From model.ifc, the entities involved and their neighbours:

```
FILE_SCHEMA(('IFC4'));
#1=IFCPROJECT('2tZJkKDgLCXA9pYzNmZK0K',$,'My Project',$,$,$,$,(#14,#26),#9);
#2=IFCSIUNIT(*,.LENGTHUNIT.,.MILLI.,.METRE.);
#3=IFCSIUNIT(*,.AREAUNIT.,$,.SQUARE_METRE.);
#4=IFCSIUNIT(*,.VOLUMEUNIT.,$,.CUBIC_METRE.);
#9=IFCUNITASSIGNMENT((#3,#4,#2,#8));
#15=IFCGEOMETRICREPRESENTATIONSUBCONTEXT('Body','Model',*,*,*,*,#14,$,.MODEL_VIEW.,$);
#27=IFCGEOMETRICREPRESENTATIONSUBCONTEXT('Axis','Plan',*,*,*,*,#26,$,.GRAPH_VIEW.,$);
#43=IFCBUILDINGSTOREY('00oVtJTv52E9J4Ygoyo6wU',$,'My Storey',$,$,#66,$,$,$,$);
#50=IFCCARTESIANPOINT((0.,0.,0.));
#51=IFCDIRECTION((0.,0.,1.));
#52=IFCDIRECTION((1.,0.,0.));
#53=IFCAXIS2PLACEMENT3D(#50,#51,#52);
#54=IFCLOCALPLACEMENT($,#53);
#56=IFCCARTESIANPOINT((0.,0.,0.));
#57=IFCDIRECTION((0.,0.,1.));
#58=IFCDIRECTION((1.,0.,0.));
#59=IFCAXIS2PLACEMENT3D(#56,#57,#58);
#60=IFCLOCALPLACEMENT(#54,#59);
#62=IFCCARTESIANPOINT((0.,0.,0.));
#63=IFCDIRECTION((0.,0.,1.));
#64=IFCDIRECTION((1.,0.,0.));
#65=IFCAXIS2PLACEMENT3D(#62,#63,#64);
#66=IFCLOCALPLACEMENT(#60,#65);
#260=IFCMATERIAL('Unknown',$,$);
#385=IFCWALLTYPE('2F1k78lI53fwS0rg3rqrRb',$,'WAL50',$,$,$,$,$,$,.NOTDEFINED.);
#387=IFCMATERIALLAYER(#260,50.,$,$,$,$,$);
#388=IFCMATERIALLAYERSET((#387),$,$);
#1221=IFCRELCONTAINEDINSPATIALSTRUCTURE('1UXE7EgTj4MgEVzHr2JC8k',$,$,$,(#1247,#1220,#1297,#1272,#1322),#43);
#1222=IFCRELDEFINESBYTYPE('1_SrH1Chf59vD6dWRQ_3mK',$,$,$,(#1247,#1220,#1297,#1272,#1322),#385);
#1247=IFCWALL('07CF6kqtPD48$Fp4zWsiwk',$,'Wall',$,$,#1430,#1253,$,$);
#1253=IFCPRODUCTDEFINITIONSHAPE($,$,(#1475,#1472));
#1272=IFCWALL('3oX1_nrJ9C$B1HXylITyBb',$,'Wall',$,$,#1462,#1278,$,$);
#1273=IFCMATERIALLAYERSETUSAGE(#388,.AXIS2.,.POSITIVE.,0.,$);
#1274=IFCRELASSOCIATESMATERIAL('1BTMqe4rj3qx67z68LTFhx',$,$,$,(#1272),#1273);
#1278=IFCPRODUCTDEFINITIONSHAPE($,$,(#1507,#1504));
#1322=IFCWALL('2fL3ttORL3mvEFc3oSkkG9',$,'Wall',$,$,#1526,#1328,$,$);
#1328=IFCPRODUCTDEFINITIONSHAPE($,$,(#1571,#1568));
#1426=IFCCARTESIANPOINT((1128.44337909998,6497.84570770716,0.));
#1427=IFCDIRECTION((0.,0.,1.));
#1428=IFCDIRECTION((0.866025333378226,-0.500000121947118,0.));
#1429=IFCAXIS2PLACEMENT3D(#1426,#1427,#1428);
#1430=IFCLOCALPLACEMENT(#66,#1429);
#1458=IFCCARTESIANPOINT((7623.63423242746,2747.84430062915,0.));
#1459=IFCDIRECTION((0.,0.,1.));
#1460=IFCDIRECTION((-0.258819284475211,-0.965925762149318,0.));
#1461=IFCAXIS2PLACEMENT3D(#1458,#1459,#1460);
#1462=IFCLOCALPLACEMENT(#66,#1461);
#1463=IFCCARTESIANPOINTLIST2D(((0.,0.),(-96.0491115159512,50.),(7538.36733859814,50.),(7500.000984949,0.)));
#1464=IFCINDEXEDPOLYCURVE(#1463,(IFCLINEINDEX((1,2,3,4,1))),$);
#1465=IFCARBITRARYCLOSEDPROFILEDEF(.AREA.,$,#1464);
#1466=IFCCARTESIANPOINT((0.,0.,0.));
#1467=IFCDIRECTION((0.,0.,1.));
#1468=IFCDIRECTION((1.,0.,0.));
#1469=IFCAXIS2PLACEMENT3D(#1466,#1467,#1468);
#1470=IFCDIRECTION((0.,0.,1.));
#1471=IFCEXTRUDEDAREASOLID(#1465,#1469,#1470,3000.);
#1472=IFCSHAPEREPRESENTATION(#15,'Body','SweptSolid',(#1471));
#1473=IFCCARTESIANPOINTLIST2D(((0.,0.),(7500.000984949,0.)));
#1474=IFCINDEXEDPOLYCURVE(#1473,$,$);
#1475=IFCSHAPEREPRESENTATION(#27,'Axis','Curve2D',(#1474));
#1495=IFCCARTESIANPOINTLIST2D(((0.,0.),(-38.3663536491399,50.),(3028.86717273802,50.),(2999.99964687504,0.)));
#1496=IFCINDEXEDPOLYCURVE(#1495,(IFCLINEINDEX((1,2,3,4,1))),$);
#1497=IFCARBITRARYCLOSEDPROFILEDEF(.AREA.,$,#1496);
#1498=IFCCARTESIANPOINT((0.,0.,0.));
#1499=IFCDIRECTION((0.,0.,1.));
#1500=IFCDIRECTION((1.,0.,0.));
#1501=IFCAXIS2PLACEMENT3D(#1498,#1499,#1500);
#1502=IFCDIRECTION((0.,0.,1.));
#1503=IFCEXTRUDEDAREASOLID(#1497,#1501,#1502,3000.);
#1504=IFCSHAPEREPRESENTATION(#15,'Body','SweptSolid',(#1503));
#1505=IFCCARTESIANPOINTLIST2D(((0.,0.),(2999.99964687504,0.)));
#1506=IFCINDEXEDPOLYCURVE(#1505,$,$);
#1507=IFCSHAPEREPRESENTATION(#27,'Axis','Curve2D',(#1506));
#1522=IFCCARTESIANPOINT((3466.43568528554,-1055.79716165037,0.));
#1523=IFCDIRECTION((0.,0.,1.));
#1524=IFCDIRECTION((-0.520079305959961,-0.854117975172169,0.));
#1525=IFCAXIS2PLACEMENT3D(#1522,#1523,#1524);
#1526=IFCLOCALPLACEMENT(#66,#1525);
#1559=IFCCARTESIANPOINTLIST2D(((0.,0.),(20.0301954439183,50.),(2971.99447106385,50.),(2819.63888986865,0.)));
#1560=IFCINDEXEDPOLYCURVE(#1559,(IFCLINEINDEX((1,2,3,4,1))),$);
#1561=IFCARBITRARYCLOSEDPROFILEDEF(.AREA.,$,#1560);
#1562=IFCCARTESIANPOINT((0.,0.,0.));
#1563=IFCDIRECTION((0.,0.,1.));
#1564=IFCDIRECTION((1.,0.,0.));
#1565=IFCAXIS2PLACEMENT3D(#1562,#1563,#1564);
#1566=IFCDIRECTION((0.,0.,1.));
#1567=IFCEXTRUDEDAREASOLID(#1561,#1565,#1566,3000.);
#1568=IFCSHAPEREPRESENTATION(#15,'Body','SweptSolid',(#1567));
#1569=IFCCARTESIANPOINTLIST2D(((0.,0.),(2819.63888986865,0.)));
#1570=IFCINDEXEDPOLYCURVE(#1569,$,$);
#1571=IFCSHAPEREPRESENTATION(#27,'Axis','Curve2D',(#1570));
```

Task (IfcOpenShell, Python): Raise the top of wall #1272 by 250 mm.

```python
import ifcopenshell
import ifcopenshell.geom
import ifcopenshell.util.representation
import ifcopenshell.util.shape
import ifcopenshell.util.unit

model = ifcopenshell.open("model.ifc")
unit_scale = ifcopenshell.util.unit.calculate_unit_scale(model)
settings = ifcopenshell.geom.settings()


def volume(element):
    """Net volume in cubic metres, openings subtracted."""
    shape = ifcopenshell.geom.create_shape(settings, element)
    return ifcopenshell.util.shape.get_volume(shape.geometry)


wall = model.by_guid("3oX1_nrJ9C$B1HXylITyBb")
before = volume(wall)

body = ifcopenshell.util.representation.get_representation(wall, "Model", "Body")
solid = body.Items[0]
old_height = solid.Depth
solid.Depth += 0.25 / unit_scale
after = volume(wall)

print(f"height {old_height:g} -> {solid.Depth:g}, volume {before:.3f} -> {after:.3f} m3")

model.write("model-out.ifc")
```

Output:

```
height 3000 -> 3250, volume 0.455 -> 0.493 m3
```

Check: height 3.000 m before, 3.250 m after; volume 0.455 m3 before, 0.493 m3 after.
